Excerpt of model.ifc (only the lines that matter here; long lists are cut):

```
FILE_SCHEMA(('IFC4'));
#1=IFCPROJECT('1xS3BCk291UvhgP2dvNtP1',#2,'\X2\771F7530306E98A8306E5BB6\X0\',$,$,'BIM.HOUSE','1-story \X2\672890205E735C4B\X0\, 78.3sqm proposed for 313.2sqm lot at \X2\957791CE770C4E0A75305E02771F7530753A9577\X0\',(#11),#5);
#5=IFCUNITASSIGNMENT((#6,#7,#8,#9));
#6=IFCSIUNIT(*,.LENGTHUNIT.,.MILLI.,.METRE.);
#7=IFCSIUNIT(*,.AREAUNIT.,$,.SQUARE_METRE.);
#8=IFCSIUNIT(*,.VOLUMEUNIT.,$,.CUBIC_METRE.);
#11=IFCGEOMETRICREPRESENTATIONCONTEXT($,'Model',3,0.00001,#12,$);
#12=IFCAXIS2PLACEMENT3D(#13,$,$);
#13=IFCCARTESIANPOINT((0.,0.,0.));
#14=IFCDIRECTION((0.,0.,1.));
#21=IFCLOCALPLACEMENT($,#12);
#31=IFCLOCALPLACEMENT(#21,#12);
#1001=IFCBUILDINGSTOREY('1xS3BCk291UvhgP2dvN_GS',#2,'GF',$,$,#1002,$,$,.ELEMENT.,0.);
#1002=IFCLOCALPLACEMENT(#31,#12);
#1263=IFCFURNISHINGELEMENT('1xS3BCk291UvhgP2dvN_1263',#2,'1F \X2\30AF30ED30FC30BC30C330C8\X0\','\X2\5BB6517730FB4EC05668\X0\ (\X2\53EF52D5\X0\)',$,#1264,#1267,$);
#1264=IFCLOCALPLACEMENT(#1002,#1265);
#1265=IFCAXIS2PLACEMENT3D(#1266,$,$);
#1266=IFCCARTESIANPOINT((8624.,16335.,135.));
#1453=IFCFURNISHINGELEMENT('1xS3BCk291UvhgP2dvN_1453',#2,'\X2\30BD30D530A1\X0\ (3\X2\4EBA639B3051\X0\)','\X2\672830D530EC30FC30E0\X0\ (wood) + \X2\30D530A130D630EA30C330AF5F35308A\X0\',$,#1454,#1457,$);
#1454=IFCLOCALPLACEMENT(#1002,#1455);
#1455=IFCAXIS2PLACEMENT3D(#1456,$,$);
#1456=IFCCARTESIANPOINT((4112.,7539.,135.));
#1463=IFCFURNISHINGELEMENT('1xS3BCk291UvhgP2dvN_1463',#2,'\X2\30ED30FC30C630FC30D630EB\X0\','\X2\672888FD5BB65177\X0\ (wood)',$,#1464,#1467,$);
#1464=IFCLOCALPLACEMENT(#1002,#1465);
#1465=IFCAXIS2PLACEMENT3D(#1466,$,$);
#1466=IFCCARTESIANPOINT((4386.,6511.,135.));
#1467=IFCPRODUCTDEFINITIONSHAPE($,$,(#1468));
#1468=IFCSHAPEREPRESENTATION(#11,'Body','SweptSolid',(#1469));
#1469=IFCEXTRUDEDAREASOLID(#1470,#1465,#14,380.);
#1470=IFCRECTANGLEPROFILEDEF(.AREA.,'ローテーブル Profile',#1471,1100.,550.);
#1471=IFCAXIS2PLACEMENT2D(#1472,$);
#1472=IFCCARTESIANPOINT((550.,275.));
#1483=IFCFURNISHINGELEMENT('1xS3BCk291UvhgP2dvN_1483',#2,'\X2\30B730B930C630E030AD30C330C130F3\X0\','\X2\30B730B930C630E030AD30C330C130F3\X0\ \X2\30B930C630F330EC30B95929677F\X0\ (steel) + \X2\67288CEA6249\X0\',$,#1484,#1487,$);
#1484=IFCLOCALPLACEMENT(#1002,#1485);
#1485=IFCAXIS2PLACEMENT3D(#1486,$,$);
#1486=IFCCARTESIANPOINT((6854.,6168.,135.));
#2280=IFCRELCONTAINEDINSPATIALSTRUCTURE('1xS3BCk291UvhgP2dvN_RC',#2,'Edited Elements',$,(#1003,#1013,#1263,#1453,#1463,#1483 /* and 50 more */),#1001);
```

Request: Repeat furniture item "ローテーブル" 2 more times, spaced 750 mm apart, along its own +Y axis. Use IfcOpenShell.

```python
import ifcopenshell
import ifcopenshell.api.geometry
import ifcopenshell.api.root
import ifcopenshell.util.element
import ifcopenshell.util.placement
import ifcopenshell.util.unit

model = ifcopenshell.open("model.ifc")
unit_scale = ifcopenshell.util.unit.calculate_unit_scale(model)


def reuse_history(source, copy):
    """copy_class also copies each property set's owner history, people and application; keep the originals."""
    for rel in copy.IsDefinedBy:
        if rel.is_a("IfcRelDefinesByProperties") and (history := rel.RelatingPropertyDefinition.OwnerHistory):
            rel.RelatingPropertyDefinition.OwnerHistory = source.OwnerHistory
            ifcopenshell.util.element.remove_deep2(model, history)


source = model.by_guid("1xS3BCk291UvhgP2dvN_1463")
base = ifcopenshell.util.placement.get_local_placement(source.ObjectPlacement)
step = base[:3, 1] * 0.75 / unit_scale

for i in range(1, 3):
    copy = ifcopenshell.api.root.copy_class(model, product=source)
    copy.Representation = ifcopenshell.util.element.copy_deep(
        model, source.Representation, exclude=["IfcGeometricRepresentationContext", "IfcRepresentationMap"]
    )
    reuse_history(source, copy)
    matrix = base.copy()
    matrix[:3, 3] += i * step
    print("added at", matrix[:3, 3].round(3) + 0.0)
    ifcopenshell.api.geometry.edit_object_placement(model, product=copy, matrix=matrix, is_si=False)

model.write("model_v2.ifc")
```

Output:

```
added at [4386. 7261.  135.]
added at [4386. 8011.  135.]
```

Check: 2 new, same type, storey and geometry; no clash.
